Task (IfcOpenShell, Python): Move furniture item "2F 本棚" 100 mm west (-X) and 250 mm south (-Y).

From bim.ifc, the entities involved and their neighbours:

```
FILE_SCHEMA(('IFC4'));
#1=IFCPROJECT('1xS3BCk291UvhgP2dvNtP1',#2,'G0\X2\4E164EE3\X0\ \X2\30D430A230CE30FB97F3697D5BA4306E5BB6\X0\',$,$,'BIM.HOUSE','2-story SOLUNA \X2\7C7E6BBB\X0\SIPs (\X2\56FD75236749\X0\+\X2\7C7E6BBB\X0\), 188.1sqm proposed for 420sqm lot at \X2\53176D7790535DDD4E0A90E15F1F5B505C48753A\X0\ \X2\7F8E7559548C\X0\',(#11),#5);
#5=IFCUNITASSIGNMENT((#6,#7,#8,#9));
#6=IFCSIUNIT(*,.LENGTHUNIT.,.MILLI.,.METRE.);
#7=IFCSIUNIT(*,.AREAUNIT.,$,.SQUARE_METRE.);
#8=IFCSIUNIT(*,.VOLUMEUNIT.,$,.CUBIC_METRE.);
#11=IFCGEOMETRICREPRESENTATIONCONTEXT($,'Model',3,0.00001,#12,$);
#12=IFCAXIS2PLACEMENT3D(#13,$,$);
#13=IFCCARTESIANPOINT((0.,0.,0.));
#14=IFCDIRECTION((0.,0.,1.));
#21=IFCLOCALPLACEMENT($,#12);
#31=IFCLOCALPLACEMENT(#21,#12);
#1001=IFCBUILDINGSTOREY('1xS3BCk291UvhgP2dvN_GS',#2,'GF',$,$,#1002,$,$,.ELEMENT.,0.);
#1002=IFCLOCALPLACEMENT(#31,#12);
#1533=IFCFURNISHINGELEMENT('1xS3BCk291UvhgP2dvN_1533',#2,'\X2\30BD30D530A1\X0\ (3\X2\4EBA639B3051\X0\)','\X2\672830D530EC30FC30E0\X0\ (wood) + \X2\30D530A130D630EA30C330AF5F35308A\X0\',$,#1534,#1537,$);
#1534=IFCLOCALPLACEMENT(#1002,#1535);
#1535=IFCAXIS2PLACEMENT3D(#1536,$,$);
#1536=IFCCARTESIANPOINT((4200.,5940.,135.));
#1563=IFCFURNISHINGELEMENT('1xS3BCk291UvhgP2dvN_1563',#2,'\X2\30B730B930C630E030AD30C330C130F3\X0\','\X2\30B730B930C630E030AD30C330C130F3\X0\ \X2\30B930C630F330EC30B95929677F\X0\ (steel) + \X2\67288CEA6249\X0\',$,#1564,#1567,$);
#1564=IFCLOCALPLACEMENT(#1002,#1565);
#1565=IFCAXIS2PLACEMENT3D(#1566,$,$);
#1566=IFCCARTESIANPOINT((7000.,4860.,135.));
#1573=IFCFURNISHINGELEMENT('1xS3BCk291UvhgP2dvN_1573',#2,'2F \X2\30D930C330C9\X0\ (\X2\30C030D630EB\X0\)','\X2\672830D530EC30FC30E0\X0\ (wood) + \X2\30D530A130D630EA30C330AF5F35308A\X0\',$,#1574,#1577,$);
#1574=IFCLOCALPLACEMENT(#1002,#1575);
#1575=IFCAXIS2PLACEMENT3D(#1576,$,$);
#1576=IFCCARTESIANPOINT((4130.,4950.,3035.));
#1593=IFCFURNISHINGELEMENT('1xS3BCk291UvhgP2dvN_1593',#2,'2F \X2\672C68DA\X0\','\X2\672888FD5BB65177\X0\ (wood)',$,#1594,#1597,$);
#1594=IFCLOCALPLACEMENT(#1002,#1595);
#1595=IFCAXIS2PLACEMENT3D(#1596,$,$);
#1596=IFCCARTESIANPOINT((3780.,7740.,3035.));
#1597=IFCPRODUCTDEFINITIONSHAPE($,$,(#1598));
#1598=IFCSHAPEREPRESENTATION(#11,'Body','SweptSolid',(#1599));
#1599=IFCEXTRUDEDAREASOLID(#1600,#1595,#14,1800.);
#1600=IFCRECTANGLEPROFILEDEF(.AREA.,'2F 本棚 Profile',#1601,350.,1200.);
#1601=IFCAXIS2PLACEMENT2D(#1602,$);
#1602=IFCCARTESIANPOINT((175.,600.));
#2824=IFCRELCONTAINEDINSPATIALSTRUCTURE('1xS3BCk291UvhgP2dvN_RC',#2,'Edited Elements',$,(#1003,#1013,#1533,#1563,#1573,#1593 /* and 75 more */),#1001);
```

```python
import ifcopenshell
import ifcopenshell.api.geometry
import ifcopenshell.util.placement
import ifcopenshell.util.unit

model = ifcopenshell.open("bim.ifc")
unit_scale = ifcopenshell.util.unit.calculate_unit_scale(model)

item = model.by_id(1593)
matrix = ifcopenshell.util.placement.get_local_placement(item.ObjectPlacement)
matrix[0, 3] -= 0.1 / unit_scale
matrix[1, 3] -= 0.25 / unit_scale
ifcopenshell.api.geometry.edit_object_placement(model, product=item, matrix=matrix, is_si=False)

print(ifcopenshell.util.placement.get_local_placement(item.ObjectPlacement).round(3) + 0.0)

model.write("bim_edited.ifc")
```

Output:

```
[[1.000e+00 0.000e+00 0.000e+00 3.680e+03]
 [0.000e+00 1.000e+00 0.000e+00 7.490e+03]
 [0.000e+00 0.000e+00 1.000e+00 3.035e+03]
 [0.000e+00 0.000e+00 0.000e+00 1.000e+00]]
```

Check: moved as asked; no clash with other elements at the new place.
